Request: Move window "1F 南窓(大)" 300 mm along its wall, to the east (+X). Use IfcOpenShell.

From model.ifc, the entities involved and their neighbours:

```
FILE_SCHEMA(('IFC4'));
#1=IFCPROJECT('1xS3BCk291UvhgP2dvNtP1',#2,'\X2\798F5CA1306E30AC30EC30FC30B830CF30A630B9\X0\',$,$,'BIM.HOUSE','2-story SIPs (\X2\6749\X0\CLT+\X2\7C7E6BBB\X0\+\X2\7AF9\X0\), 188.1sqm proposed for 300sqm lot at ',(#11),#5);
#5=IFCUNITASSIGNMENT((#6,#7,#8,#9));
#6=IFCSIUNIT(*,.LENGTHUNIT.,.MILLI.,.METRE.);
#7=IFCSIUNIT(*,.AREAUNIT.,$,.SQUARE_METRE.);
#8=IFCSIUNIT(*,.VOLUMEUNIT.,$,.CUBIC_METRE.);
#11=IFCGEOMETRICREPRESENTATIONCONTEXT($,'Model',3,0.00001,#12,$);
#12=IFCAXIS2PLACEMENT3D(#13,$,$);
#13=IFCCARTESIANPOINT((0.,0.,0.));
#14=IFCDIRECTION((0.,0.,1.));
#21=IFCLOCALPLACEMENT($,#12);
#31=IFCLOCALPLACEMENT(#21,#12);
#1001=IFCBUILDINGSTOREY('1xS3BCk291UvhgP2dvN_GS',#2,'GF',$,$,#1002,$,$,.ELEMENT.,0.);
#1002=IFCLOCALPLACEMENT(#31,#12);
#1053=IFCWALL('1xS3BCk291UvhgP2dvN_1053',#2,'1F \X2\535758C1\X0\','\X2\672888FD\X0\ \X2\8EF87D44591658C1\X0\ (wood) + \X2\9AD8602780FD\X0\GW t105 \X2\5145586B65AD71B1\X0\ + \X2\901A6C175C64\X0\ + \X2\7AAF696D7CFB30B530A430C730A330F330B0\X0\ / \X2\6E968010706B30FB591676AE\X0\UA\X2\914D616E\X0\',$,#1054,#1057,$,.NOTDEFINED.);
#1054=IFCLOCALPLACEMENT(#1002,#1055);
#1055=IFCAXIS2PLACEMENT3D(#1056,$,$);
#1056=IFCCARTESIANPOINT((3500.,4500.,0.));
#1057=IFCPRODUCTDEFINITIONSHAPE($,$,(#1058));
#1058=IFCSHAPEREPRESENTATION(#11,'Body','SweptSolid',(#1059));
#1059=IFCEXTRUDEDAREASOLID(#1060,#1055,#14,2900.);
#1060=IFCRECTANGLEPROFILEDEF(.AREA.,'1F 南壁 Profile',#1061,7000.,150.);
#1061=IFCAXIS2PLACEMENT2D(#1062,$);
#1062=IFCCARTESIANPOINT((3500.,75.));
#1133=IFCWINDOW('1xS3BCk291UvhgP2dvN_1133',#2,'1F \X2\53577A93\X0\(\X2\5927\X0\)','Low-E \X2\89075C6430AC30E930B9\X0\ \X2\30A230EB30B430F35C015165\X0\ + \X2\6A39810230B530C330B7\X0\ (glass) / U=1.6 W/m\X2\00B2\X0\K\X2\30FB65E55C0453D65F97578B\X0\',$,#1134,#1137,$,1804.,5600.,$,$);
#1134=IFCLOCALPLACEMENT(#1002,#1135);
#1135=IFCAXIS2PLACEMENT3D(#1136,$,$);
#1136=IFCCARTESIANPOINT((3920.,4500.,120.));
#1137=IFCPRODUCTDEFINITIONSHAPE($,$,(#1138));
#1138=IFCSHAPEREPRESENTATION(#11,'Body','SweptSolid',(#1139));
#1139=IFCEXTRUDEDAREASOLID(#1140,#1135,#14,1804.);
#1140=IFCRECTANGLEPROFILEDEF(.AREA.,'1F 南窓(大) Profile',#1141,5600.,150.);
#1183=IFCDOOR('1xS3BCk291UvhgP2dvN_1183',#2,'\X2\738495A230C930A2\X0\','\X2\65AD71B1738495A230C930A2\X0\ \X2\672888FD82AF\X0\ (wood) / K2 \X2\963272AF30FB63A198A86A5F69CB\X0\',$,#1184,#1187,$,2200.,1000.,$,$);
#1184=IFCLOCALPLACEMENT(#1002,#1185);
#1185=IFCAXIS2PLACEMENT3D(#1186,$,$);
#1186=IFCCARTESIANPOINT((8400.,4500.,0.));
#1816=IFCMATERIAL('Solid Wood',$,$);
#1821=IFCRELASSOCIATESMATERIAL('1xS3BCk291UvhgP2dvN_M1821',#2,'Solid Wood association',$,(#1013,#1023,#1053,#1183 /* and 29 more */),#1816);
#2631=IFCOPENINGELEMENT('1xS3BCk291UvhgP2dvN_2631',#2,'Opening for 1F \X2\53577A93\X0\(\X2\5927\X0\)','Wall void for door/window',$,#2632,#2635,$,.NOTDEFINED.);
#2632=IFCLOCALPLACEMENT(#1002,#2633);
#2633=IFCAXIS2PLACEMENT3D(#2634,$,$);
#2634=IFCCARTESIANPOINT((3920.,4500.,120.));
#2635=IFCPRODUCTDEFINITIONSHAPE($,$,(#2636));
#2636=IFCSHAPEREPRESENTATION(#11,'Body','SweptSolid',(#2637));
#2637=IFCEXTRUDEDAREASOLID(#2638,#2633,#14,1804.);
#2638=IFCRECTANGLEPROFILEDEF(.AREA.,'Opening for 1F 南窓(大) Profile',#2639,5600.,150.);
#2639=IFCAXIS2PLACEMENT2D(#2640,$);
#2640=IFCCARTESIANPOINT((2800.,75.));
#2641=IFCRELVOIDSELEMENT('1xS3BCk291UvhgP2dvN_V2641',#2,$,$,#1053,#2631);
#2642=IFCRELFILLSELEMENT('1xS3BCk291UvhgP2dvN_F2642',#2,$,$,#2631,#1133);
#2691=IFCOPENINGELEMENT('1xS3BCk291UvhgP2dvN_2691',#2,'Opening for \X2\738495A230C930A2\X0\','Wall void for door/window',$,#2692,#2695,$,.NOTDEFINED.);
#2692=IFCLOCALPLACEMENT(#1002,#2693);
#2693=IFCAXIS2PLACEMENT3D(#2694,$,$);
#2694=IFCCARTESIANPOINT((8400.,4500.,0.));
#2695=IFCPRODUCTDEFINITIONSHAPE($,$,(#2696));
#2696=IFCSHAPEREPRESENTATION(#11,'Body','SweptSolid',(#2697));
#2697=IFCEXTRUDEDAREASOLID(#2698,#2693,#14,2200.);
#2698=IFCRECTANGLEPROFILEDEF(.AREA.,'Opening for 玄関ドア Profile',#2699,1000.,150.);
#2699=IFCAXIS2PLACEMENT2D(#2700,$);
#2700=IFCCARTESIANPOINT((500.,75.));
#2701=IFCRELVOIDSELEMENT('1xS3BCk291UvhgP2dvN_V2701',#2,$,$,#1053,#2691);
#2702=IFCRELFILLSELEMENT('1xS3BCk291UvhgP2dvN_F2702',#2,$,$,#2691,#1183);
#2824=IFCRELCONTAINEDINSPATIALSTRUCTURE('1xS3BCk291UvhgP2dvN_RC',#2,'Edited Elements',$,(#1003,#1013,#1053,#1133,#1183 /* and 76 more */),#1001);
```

```python
import ifcopenshell
import ifcopenshell.api.geometry
import ifcopenshell.util.placement

model = ifcopenshell.open("model.ifc")

window = model.by_id(1133)
opening = window.FillsVoids[0].RelatingOpeningElement
wall = opening.VoidsElements[0].RelatingBuildingElement

wall_matrix = ifcopenshell.util.placement.get_local_placement(wall.ObjectPlacement)
shift = wall_matrix[:3, 0] * 300.0
before = ifcopenshell.util.placement.get_local_placement(window.ObjectPlacement)[:3, 3].copy()

# The window is not placed relative to its opening, so move both.
for product in (opening, window):
    matrix = ifcopenshell.util.placement.get_local_placement(product.ObjectPlacement)
    matrix[:3, 3] += shift
    ifcopenshell.api.geometry.edit_object_placement(model, product=product, matrix=matrix, is_si=False)

after = ifcopenshell.util.placement.get_local_placement(window.ObjectPlacement)[:3, 3]
print("window moved by", (after - before).round(3) + 0.0)

model.write("model-out.ifc")
```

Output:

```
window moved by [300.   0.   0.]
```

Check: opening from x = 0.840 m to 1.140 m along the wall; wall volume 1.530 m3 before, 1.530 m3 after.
